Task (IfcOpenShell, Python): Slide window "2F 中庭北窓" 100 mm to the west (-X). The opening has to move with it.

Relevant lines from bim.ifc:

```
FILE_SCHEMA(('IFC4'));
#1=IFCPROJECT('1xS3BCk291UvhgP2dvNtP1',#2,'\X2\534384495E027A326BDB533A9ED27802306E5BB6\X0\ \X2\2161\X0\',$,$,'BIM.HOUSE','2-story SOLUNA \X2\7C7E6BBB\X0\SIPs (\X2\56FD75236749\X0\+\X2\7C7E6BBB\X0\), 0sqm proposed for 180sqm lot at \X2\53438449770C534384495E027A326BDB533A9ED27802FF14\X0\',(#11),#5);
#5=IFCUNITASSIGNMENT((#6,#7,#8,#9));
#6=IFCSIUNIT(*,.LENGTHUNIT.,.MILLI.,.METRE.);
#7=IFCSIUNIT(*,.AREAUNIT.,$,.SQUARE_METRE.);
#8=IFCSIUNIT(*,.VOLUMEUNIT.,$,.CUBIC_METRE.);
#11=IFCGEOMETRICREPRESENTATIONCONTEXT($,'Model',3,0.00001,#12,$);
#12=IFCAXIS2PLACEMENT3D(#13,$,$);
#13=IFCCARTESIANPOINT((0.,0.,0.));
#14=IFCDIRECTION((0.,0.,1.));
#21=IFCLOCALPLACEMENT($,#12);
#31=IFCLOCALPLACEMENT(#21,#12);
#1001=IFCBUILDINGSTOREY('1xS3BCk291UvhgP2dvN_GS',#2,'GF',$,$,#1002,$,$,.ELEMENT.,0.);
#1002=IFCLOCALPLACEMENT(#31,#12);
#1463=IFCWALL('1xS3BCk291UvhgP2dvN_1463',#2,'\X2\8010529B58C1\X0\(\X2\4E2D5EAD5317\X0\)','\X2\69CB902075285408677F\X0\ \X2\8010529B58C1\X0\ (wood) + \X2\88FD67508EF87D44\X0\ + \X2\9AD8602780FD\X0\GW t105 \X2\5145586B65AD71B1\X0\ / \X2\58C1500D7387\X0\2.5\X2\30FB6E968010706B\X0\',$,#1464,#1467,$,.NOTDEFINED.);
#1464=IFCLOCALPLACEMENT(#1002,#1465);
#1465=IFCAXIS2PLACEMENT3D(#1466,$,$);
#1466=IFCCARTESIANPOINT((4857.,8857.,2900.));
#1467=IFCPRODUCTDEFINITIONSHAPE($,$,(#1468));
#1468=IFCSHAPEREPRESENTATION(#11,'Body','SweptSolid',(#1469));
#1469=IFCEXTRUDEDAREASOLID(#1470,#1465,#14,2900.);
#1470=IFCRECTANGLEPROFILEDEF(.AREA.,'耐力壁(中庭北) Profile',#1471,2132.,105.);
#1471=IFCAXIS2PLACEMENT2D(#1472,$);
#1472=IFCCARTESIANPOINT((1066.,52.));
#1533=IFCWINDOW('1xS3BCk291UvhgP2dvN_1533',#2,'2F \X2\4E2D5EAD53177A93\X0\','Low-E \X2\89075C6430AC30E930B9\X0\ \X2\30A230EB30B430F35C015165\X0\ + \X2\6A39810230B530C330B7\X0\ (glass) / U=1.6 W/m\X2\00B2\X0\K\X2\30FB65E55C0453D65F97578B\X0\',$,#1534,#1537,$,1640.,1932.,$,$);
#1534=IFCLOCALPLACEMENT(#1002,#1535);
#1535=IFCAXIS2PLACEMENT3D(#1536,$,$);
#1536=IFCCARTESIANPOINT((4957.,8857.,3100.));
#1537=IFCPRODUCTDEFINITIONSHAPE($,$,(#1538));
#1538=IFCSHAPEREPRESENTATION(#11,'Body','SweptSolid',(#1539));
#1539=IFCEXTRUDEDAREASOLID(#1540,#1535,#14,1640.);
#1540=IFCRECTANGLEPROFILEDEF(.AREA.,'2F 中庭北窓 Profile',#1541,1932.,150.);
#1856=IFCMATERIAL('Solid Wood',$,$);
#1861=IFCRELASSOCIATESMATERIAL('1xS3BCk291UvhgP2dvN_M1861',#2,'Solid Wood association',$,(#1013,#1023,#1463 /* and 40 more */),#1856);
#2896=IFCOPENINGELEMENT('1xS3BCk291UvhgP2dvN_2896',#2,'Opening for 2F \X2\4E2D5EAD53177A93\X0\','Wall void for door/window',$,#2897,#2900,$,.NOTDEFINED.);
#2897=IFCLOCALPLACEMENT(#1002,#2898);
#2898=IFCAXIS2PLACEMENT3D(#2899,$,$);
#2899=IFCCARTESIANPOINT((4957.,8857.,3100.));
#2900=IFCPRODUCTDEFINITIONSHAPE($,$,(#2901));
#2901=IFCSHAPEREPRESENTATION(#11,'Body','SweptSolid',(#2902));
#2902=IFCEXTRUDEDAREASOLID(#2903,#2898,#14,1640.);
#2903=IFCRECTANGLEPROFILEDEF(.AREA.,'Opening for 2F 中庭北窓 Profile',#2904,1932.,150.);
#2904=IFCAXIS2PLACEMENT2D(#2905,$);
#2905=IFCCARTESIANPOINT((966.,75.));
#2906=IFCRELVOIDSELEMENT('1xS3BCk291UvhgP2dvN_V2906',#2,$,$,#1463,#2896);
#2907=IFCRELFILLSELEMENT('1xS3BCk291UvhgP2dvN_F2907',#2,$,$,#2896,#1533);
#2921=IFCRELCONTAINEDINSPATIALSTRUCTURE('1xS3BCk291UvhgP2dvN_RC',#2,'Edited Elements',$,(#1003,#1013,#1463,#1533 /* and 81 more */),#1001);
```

```python
import ifcopenshell
import ifcopenshell.api.geometry
import ifcopenshell.util.placement
import ifcopenshell.util.unit

model = ifcopenshell.open("bim.ifc")
unit_scale = ifcopenshell.util.unit.calculate_unit_scale(model)

window = model.by_guid("1xS3BCk291UvhgP2dvN_1533")
opening = window.FillsVoids[0].RelatingOpeningElement
wall = opening.VoidsElements[0].RelatingBuildingElement

wall_matrix = ifcopenshell.util.placement.get_local_placement(wall.ObjectPlacement)
shift = wall_matrix[:3, 0] * -0.1 / unit_scale
before = ifcopenshell.util.placement.get_local_placement(window.ObjectPlacement)[:3, 3].copy()

# The window is not placed relative to its opening, so move both.
for product in (opening, window):
    matrix = ifcopenshell.util.placement.get_local_placement(product.ObjectPlacement)
    matrix[:3, 3] += shift
    ifcopenshell.api.geometry.edit_object_placement(model, product=product, matrix=matrix, is_si=False)

after = ifcopenshell.util.placement.get_local_placement(window.ObjectPlacement)[:3, 3]
print("window moved by", (after - before).round(3) + 0.0)

model.write("bim_updated.ifc")
```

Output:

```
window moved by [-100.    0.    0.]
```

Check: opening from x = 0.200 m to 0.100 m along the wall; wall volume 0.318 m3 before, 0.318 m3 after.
